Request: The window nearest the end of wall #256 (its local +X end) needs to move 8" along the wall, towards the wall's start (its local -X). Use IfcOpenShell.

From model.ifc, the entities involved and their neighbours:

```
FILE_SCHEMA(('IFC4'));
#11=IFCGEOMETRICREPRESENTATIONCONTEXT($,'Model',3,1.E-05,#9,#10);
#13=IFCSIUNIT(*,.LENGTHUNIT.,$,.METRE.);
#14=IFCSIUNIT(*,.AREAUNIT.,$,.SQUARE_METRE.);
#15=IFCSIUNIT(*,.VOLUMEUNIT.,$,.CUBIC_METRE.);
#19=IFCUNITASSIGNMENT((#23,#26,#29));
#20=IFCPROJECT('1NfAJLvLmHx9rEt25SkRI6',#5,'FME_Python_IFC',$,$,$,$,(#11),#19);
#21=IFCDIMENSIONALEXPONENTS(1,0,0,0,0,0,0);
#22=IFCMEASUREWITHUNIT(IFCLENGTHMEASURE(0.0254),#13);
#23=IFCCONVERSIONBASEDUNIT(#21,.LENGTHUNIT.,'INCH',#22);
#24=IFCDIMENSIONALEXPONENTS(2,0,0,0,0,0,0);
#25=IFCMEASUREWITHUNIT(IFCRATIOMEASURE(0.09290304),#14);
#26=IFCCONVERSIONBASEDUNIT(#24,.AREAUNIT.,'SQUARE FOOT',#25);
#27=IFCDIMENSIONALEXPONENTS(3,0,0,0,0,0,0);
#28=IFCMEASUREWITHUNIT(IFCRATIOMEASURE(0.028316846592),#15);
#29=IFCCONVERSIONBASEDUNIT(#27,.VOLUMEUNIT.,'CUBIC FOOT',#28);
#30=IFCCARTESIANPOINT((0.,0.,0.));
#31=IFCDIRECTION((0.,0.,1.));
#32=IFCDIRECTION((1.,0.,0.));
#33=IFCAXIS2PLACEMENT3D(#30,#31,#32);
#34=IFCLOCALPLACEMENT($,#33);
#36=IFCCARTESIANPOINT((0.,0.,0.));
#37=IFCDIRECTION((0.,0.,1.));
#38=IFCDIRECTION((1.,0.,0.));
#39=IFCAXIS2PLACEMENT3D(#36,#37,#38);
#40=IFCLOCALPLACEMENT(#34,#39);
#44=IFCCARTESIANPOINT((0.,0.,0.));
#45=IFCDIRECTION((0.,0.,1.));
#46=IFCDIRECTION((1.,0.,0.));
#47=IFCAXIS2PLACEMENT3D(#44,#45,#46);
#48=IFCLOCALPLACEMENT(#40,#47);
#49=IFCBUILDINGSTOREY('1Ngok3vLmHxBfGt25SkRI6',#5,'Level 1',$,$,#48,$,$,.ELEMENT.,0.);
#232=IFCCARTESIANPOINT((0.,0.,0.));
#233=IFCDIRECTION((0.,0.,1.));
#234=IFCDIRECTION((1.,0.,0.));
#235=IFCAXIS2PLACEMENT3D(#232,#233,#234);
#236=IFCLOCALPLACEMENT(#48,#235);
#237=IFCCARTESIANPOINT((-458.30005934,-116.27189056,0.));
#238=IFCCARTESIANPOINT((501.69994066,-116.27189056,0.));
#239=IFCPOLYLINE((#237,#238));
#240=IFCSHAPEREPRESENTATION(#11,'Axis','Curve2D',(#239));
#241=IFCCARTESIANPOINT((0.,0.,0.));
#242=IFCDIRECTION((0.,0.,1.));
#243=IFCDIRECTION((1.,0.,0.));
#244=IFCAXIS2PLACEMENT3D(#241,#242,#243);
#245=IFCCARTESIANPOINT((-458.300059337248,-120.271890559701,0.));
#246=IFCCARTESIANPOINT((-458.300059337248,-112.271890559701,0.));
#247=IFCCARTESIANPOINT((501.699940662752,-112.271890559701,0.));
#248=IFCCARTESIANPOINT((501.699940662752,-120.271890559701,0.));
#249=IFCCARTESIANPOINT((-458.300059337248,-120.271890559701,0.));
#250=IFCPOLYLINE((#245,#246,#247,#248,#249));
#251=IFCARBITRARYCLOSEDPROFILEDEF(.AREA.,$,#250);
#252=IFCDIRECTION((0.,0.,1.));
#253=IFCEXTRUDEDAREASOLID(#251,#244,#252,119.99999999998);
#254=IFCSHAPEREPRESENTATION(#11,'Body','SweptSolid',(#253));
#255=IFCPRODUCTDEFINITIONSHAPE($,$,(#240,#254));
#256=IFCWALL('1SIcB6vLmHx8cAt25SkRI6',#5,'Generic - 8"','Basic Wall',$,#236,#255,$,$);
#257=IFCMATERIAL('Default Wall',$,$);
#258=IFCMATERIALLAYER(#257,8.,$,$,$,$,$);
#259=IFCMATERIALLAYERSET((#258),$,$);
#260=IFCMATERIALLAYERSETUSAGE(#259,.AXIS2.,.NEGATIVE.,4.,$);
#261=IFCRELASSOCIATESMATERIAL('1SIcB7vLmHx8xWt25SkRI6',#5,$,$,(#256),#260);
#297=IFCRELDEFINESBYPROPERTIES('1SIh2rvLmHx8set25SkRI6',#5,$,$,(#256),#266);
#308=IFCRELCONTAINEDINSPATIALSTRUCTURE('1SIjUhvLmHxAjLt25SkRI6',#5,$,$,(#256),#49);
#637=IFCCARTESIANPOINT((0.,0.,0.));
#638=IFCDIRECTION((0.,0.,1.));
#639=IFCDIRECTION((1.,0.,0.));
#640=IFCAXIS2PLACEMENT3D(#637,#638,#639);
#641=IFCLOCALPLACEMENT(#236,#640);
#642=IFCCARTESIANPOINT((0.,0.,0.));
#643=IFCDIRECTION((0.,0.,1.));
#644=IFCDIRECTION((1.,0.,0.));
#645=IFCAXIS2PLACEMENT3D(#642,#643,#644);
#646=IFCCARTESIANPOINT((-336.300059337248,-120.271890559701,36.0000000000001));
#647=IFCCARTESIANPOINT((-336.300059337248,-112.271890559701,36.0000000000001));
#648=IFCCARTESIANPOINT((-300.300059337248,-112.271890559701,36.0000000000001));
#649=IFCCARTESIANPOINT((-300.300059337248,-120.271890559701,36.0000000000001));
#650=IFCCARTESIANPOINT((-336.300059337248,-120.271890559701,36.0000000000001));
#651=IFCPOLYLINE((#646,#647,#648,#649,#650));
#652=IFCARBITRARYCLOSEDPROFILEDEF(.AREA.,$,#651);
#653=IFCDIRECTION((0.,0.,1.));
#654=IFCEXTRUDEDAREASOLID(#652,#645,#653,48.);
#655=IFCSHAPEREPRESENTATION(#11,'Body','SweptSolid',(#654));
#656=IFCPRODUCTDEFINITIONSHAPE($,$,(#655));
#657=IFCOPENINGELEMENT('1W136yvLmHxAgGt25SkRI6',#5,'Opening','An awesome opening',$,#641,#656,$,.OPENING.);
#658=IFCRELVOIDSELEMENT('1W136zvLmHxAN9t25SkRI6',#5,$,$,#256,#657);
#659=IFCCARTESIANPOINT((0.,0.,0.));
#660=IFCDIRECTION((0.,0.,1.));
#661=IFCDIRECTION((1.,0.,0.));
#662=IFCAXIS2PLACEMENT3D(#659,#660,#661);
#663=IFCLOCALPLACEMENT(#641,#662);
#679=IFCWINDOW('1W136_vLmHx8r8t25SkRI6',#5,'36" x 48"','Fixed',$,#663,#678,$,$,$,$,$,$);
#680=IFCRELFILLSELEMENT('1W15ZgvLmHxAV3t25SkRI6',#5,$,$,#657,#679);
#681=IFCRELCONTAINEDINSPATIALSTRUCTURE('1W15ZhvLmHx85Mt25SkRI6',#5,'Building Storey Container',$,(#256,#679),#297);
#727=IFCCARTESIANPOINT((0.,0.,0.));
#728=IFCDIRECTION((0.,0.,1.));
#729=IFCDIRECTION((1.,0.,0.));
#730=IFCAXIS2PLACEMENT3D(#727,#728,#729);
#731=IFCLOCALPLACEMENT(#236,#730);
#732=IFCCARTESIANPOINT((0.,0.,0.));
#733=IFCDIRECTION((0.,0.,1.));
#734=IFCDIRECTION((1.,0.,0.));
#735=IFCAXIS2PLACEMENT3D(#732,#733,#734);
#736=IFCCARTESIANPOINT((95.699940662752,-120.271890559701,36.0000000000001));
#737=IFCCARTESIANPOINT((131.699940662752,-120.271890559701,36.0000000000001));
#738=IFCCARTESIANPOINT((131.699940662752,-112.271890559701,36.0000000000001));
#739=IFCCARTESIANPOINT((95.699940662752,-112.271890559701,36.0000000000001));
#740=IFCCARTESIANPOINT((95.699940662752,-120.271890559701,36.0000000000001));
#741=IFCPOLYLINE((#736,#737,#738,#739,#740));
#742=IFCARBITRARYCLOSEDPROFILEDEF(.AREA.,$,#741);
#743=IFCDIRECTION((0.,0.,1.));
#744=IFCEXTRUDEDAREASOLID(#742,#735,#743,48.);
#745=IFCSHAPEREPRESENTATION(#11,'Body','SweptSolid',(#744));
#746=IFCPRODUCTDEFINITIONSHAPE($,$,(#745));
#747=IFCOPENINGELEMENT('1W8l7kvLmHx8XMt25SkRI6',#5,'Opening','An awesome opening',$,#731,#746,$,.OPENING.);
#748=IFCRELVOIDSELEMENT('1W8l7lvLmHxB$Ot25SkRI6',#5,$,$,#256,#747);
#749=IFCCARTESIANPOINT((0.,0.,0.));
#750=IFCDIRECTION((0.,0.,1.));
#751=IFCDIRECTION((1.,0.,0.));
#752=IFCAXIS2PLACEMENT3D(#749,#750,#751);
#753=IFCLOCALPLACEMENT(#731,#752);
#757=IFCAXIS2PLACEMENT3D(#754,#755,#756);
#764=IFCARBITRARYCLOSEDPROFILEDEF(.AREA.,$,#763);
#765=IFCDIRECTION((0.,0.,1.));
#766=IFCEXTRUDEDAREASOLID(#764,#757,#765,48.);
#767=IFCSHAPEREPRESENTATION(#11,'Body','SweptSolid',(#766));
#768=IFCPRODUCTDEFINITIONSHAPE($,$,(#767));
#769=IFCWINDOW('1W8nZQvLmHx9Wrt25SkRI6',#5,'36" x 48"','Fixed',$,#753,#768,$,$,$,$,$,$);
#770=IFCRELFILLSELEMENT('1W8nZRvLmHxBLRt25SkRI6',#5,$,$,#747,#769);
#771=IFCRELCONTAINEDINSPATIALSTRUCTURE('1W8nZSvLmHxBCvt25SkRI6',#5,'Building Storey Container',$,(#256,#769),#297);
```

```python
import ifcopenshell
import ifcopenshell.api.geometry
import ifcopenshell.util.placement
import ifcopenshell.util.unit

model = ifcopenshell.open("model.ifc")
unit_scale = ifcopenshell.util.unit.calculate_unit_scale(model)

window = model.by_guid("1W8nZQvLmHx9Wrt25SkRI6")
opening = window.FillsVoids[0].RelatingOpeningElement
wall = opening.VoidsElements[0].RelatingBuildingElement

wall_matrix = ifcopenshell.util.placement.get_local_placement(wall.ObjectPlacement)
shift = wall_matrix[:3, 0] * -8 * 0.0254 / unit_scale
before = ifcopenshell.util.placement.get_local_placement(window.ObjectPlacement)[:3, 3].copy()

# The window is placed relative to its opening, so it follows when the opening moves.
matrix = ifcopenshell.util.placement.get_local_placement(opening.ObjectPlacement)
matrix[:3, 3] += shift
ifcopenshell.api.geometry.edit_object_placement(
    model, product=opening, matrix=matrix, is_si=False, should_transform_children=True
)

after = ifcopenshell.util.placement.get_local_placement(window.ObjectPlacement)[:3, 3]
print("window moved by", (after - before).round(3) + 0.0)

model.write("model_edited.ifc")
```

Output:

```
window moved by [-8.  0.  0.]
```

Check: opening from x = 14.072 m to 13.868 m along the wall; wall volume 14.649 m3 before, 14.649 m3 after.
